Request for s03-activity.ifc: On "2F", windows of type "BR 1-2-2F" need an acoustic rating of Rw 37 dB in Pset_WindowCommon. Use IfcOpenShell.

First a look at what the model holds.

```python
import ifcopenshell
import ifcopenshell.util.element

model = ifcopenshell.open("s03-activity.ifc")
print(model.schema)
storey = next(s for s in model.by_type("IfcBuildingStorey") if s.Name == "2F")
windows = [e for e in ifcopenshell.util.element.get_decomposition(storey) if e.is_a("IfcWindow")]
seen = {}
for e in windows:
    element_type = ifcopenshell.util.element.get_type(e)
    key = (element_type.Name if element_type != e and element_type else None, ifcopenshell.util.element.get_pset(e, "Pset_WindowCommon", "AcousticRating"))
    seen[key] = seen.get(key, 0) + 1
for (name, value), count in sorted(seen.items(), key=str):
    print(count, "x", name, "|", value)
```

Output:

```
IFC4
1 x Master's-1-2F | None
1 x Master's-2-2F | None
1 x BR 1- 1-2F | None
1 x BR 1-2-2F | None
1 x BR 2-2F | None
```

```python
import ifcopenshell
import ifcopenshell.api.pset
import ifcopenshell.util.element

model = ifcopenshell.open("s03-activity.ifc")

storey = next(s for s in model.by_type("IfcBuildingStorey") if s.Name == "2F")
windows = [e for e in ifcopenshell.util.element.get_decomposition(storey) if e.is_a("IfcWindow")]

count = 0
for e in windows:
    element_type = ifcopenshell.util.element.get_type(e)
    if element_type in (None, e) or element_type.Name != "BR 1-2-2F":
        continue
    # add_pset returns the element's existing set when there is one.
    pset = ifcopenshell.api.pset.add_pset(model, product=e, name="Pset_WindowCommon")
    ifcopenshell.api.pset.edit_pset(model, pset=pset, properties={"AcousticRating": "Rw 37 dB"})
    count += 1

print(count, "windows updated")

model.write("s03-activity_rev.ifc")
```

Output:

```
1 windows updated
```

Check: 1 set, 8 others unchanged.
